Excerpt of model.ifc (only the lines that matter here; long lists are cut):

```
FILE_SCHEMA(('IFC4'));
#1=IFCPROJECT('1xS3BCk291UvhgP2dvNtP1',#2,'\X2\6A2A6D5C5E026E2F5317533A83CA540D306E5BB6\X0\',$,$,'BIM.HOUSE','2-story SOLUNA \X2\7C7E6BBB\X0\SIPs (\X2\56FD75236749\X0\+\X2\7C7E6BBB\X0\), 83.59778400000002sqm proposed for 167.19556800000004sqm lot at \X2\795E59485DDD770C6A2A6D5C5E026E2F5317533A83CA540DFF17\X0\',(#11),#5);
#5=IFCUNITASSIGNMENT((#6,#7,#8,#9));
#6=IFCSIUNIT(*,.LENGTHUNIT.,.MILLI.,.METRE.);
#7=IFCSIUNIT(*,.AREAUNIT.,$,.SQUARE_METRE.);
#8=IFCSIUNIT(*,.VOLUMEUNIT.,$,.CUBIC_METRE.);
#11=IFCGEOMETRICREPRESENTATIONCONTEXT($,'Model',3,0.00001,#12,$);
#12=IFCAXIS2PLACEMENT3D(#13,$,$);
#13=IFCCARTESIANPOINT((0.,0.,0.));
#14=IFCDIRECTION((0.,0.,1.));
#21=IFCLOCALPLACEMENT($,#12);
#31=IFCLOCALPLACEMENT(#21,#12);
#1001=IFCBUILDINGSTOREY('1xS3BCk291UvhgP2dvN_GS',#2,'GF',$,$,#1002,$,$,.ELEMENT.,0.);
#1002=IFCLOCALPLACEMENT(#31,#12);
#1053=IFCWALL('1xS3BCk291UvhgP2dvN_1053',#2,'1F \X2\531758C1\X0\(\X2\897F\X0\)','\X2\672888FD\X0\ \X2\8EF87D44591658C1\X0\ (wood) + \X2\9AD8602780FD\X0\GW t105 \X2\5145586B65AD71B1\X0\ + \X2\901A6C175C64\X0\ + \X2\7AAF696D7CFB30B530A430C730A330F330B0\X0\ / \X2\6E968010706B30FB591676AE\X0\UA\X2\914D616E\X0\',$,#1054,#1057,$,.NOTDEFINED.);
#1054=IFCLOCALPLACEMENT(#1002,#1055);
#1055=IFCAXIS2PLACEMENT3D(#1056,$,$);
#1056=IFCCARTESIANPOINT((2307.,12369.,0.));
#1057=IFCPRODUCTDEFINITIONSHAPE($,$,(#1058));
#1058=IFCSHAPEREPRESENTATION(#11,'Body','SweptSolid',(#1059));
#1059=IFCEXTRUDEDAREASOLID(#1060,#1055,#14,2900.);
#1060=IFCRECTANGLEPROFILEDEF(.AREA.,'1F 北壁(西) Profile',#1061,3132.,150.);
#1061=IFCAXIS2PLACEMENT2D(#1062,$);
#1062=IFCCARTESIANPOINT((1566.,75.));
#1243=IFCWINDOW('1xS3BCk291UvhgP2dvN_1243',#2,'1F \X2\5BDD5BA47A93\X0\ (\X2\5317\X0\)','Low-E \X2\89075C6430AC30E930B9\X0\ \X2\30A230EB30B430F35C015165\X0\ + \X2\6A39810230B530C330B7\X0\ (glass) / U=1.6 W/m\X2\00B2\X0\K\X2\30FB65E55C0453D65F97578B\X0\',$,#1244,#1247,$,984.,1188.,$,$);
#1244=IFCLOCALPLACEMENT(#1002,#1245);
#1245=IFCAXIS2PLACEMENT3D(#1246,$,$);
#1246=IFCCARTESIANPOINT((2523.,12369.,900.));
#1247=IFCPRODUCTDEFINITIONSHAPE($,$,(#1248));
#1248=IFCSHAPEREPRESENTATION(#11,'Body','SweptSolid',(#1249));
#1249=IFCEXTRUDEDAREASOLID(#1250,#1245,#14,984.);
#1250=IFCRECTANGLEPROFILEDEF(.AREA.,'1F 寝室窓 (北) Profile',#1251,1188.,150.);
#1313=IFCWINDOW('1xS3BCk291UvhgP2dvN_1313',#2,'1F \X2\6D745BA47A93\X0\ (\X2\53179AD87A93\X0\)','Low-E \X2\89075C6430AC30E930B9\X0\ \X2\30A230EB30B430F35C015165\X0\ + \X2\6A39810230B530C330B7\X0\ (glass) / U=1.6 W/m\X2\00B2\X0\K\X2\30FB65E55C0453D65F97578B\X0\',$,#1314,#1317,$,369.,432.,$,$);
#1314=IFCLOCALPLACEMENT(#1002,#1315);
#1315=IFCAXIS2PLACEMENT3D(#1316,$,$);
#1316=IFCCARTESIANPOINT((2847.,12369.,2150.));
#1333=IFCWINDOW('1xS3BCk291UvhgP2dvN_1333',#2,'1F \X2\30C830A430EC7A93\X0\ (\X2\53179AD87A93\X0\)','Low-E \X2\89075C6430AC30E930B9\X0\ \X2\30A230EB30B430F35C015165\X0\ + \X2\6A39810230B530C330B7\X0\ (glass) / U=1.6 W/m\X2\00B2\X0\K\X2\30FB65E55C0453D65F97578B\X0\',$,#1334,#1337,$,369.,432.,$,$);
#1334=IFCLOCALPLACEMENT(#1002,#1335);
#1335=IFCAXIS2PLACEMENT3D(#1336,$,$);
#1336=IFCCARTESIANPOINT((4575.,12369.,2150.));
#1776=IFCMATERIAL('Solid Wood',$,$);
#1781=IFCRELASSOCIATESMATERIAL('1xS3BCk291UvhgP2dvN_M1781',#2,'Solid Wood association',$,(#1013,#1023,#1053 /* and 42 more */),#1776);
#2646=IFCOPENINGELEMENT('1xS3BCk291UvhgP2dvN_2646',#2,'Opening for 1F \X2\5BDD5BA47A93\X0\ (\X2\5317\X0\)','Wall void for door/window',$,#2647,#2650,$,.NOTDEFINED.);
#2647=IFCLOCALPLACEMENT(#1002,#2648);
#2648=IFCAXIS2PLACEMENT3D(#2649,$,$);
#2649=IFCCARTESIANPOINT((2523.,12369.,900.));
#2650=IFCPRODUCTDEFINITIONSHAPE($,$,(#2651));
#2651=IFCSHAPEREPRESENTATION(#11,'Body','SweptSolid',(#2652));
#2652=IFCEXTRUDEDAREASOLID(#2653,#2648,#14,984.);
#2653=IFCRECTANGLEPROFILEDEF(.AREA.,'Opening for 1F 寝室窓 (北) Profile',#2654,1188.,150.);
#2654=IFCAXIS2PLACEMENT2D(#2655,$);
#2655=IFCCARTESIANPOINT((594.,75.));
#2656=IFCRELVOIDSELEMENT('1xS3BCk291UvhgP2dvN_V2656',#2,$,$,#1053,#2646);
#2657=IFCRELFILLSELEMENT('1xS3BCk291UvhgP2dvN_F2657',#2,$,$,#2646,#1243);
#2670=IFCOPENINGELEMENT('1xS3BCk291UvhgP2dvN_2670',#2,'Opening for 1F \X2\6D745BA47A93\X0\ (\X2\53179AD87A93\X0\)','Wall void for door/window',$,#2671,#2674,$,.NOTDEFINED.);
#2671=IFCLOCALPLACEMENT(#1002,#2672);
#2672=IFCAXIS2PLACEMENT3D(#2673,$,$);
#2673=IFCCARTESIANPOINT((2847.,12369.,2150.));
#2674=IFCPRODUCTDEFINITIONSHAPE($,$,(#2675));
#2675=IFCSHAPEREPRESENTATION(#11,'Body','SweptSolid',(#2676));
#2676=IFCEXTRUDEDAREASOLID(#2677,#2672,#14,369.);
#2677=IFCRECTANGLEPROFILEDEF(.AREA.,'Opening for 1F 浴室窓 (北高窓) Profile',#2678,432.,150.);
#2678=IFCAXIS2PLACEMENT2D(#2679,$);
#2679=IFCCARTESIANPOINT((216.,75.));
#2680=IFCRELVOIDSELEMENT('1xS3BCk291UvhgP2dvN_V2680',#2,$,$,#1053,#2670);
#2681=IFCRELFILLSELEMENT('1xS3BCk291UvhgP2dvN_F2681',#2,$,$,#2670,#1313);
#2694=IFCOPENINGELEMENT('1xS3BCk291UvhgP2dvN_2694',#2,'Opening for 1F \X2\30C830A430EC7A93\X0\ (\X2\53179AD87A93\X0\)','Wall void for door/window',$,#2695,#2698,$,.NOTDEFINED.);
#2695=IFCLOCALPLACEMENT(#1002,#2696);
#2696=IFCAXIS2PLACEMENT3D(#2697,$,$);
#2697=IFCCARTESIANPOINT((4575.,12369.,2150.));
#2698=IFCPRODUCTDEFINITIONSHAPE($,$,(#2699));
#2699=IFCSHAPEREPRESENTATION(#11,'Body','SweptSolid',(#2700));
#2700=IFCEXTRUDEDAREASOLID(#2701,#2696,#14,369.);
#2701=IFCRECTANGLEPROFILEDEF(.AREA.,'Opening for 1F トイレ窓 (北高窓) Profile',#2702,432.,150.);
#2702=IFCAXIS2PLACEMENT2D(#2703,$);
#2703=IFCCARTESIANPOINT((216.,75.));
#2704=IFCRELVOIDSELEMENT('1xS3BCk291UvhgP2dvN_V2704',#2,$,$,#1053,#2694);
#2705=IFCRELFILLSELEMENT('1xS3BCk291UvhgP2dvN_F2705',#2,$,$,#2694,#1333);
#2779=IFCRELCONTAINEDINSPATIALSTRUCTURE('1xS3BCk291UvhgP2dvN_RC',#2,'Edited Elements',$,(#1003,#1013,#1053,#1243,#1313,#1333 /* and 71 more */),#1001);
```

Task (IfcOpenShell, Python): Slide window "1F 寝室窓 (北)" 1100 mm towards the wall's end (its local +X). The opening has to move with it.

```python
import ifcopenshell
import ifcopenshell.api.geometry
import ifcopenshell.util.placement

model = ifcopenshell.open("model.ifc")

window = model.by_id(1243)
opening = window.FillsVoids[0].RelatingOpeningElement
wall = opening.VoidsElements[0].RelatingBuildingElement

wall_matrix = ifcopenshell.util.placement.get_local_placement(wall.ObjectPlacement)
shift = wall_matrix[:3, 0] * 1100.0
before = ifcopenshell.util.placement.get_local_placement(window.ObjectPlacement)[:3, 3].copy()

# The window is not placed relative to its opening, so move both.
for product in (opening, window):
    matrix = ifcopenshell.util.placement.get_local_placement(product.ObjectPlacement)
    matrix[:3, 3] += shift
    ifcopenshell.api.geometry.edit_object_placement(model, product=product, matrix=matrix, is_si=False)

after = ifcopenshell.util.placement.get_local_placement(window.ObjectPlacement)[:3, 3]
print("window moved by", (after - before).round(3) + 0.0)

model.write("model_rev.ifc")
```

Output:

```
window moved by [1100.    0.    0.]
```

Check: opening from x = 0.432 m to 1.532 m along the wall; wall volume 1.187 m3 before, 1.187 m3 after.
